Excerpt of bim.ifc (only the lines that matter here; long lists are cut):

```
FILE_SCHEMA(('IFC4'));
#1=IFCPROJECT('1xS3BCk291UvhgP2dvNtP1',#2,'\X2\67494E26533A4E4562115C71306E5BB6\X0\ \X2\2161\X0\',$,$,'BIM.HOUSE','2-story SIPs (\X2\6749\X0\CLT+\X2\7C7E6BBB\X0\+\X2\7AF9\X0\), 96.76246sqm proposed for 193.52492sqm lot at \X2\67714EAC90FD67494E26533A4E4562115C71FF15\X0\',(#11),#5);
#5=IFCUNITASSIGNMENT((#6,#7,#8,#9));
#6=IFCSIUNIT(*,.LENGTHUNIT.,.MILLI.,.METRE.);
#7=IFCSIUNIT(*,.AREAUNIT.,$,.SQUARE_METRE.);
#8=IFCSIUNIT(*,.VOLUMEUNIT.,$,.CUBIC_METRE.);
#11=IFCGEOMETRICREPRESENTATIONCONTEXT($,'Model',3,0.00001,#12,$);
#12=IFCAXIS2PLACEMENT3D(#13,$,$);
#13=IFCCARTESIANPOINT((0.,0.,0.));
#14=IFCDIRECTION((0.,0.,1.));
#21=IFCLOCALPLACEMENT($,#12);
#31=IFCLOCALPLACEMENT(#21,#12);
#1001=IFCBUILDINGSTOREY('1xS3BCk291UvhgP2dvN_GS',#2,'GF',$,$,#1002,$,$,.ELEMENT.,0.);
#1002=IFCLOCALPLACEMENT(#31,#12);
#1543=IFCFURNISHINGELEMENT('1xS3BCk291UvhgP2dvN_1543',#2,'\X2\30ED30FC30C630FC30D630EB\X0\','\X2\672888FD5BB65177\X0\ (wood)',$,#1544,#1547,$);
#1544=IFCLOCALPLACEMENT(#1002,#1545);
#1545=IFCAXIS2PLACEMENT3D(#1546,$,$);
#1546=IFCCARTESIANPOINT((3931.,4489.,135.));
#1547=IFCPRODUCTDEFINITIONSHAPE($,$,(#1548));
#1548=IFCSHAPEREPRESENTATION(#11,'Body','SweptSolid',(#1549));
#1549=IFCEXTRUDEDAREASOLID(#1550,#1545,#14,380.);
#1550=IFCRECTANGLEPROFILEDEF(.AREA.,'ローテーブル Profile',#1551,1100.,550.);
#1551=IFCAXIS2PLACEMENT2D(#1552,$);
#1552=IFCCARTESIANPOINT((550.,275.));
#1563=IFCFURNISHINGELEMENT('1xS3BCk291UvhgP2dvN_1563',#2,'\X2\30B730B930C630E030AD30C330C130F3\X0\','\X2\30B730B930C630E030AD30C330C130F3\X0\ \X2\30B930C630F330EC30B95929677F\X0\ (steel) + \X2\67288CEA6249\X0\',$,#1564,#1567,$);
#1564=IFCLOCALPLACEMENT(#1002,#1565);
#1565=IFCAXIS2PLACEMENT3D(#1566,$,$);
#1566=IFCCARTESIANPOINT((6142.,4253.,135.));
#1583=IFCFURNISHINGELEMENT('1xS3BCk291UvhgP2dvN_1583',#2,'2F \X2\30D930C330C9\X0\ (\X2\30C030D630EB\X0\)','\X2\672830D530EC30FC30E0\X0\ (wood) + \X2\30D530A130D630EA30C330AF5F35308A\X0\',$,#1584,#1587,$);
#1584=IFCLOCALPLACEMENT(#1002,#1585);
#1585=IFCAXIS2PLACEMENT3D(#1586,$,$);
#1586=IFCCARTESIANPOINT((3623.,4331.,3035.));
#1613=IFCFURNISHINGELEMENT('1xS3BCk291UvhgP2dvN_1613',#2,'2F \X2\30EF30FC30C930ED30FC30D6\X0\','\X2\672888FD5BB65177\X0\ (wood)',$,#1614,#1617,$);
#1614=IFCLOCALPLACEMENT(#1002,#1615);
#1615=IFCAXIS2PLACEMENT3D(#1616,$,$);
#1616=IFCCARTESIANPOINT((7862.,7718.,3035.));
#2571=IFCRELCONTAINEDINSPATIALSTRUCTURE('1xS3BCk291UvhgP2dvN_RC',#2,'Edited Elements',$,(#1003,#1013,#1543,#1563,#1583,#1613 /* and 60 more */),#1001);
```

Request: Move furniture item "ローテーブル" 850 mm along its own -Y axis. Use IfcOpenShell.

```python
import ifcopenshell
import ifcopenshell.api.geometry
import ifcopenshell.util.placement
import ifcopenshell.util.unit

model = ifcopenshell.open("bim.ifc")
unit_scale = ifcopenshell.util.unit.calculate_unit_scale(model)

item = model.by_guid("1xS3BCk291UvhgP2dvN_1543")
matrix = ifcopenshell.util.placement.get_local_placement(item.ObjectPlacement)
matrix[:3, 3] -= matrix[:3, 1] * 0.85 / unit_scale
ifcopenshell.api.geometry.edit_object_placement(model, product=item, matrix=matrix, is_si=False)

print(ifcopenshell.util.placement.get_local_placement(item.ObjectPlacement).round(3) + 0.0)

model.write("bim_edited.ifc")
```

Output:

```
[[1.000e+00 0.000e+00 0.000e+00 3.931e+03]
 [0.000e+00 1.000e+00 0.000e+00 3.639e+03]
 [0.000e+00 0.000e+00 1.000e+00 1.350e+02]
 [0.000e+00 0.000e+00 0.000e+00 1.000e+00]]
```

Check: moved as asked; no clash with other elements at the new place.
